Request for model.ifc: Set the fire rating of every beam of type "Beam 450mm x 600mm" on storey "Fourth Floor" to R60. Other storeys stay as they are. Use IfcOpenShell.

First a look at what the model holds.

```python
import ifcopenshell
import ifcopenshell.util.element

model = ifcopenshell.open("model.ifc")
print(model.schema)
storey = next(s for s in model.by_type("IfcBuildingStorey") if s.Name == "Fourth Floor")
beams = [e for e in ifcopenshell.util.element.get_decomposition(storey) if e.is_a("IfcBeam")]
seen = {}
for e in beams:
    element_type = ifcopenshell.util.element.get_type(e)
    key = (element_type.Name if element_type != e and element_type else None, ifcopenshell.util.element.get_pset(e, "Pset_BeamCommon", "FireRating"))
    seen[key] = seen.get(key, 0) + 1
for (name, value), count in sorted(seen.items(), key=str):
    print(count, "x", name, "|", value)
```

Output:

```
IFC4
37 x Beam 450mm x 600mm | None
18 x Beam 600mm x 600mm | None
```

```python
import ifcopenshell
import ifcopenshell.api.pset
import ifcopenshell.util.element

model = ifcopenshell.open("model.ifc")

storey = next(s for s in model.by_type("IfcBuildingStorey") if s.Name == "Fourth Floor")
beams = [e for e in ifcopenshell.util.element.get_decomposition(storey) if e.is_a("IfcBeam")]

count = 0
for e in beams:
    element_type = ifcopenshell.util.element.get_type(e)
    if element_type in (None, e) or element_type.Name != "Beam 450mm x 600mm":
        continue
    # add_pset returns the element's existing set when there is one.
    pset = ifcopenshell.api.pset.add_pset(model, product=e, name="Pset_BeamCommon")
    ifcopenshell.api.pset.edit_pset(model, pset=pset, properties={"FireRating": "R60"})
    count += 1

print(count, "beams updated")

model.write("model_rev.ifc")
```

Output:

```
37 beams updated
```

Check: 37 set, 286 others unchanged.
